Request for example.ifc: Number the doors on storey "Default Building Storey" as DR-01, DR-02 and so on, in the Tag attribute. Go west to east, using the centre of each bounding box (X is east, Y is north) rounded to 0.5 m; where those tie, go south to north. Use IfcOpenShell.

First a look at what the model holds.

```python
import ifcopenshell
import ifcopenshell.util.element
import ifcopenshell.util.placement

model = ifcopenshell.open("example.ifc")
print(model.schema)
storey = next(s for s in model.by_type("IfcBuildingStorey") if s.Name == "Default Building Storey")
doors = [e for e in ifcopenshell.util.element.get_decomposition(storey) if e.is_a("IfcDoor")]
for e in sorted(doors, key=lambda e: e.id()):
    origin = ifcopenshell.util.placement.get_local_placement(e.ObjectPlacement)[:3, 3]
    print(e.id(), e.Tag, e.Name, origin.round(2) + 0.0, sep=" | ")
```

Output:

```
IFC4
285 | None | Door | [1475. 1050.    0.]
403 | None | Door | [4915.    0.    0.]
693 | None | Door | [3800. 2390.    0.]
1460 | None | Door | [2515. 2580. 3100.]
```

```python
import ifcopenshell
import ifcopenshell.geom
import ifcopenshell.util.element
import ifcopenshell.util.shape

model = ifcopenshell.open("example.ifc")
settings = ifcopenshell.geom.settings()
settings.set("use-world-coords", True)


def centre(element):
    shape = ifcopenshell.geom.create_shape(settings, element)
    return ifcopenshell.util.shape.get_bbox_centroid(shape.geometry)


storey = next(s for s in model.by_type("IfcBuildingStorey") if s.Name == "Default Building Storey")
doors = [e for e in ifcopenshell.util.element.get_decomposition(storey) if e.is_a("IfcDoor")]

# Insertion points can sit at a corner or the storey origin, so sort by the geometry (in metres).
centres = {e: centre(e) for e in doors}
doors.sort(key=lambda e: (round(centres[e][0] / 0.5), centres[e][1]))

for i, e in enumerate(doors, start=1):
    number = f"DR-{i:02d}"
    e.Tag = number
    print(e.id(), number)

model.write("example_updated.ifc")
```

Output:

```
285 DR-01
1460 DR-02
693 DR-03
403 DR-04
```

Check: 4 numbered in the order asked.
